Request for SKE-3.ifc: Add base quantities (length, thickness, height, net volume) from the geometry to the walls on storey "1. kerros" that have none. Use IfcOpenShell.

First a look at what the model holds.

```python
import ifcopenshell
import ifcopenshell.util.element
import ifcopenshell.util.unit

model = ifcopenshell.open("SKE-3.ifc")
print(model.schema)
for unit_type in ("LENGTHUNIT", "AREAUNIT", "VOLUMEUNIT"):
    print(unit_type, ifcopenshell.util.unit.calculate_unit_scale(model, unit_type))
storey = next(s for s in model.by_type("IfcBuildingStorey") if s.Name == "1. kerros")
walls = [e for e in ifcopenshell.util.element.get_decomposition(storey) if e.is_a("IfcWall")]
for e in sorted(walls, key=lambda e: e.id()):
    print(e.id(), e.is_a(), e.Name, list(ifcopenshell.util.element.get_psets(e, qtos_only=True)), sep=" | ")
```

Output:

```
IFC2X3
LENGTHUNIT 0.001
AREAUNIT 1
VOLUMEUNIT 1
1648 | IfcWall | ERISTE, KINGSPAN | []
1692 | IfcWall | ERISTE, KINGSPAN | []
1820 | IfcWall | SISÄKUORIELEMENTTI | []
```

```python
import ifcopenshell
import ifcopenshell.api.pset
import ifcopenshell.geom
import ifcopenshell.util.element
import ifcopenshell.util.shape
import ifcopenshell.util.unit

model = ifcopenshell.open("SKE-3.ifc")
unit_scale = ifcopenshell.util.unit.calculate_unit_scale(model)
volume_scale = ifcopenshell.util.unit.calculate_unit_scale(model, "VOLUMEUNIT")
settings = ifcopenshell.geom.settings()

storey = next(s for s in model.by_type("IfcBuildingStorey") if s.Name == "1. kerros")
walls = [e for e in ifcopenshell.util.element.get_decomposition(storey) if e.is_a("IfcWall")]

for e in sorted(walls, key=lambda e: e.id()):
    if ifcopenshell.util.element.get_psets(e, qtos_only=True, should_inherit=False):
        continue
    # Geometry comes back in metres, in the element's own axes.
    shape = ifcopenshell.geom.create_shape(settings, e)
    values = {
        "Length": ifcopenshell.util.shape.get_x(shape.geometry) / unit_scale,
        "Width": ifcopenshell.util.shape.get_y(shape.geometry) / unit_scale,
        "Height": ifcopenshell.util.shape.get_z(shape.geometry) / unit_scale,
        "NetVolume": ifcopenshell.util.shape.get_volume(shape.geometry) / volume_scale,
    }
    qto = ifcopenshell.api.pset.add_qto(model, product=e, name="BaseQuantities")
    ifcopenshell.api.pset.edit_qto(model, qto=qto, properties=values)
    print(e.id(), {k: round(v, 3) for k, v in values.items()})

model.write("SKE-3_updated.ifc")
```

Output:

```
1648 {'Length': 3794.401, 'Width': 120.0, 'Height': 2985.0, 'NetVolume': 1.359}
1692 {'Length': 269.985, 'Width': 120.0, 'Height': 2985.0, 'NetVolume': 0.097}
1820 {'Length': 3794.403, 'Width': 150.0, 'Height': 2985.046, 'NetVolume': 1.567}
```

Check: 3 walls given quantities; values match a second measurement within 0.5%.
